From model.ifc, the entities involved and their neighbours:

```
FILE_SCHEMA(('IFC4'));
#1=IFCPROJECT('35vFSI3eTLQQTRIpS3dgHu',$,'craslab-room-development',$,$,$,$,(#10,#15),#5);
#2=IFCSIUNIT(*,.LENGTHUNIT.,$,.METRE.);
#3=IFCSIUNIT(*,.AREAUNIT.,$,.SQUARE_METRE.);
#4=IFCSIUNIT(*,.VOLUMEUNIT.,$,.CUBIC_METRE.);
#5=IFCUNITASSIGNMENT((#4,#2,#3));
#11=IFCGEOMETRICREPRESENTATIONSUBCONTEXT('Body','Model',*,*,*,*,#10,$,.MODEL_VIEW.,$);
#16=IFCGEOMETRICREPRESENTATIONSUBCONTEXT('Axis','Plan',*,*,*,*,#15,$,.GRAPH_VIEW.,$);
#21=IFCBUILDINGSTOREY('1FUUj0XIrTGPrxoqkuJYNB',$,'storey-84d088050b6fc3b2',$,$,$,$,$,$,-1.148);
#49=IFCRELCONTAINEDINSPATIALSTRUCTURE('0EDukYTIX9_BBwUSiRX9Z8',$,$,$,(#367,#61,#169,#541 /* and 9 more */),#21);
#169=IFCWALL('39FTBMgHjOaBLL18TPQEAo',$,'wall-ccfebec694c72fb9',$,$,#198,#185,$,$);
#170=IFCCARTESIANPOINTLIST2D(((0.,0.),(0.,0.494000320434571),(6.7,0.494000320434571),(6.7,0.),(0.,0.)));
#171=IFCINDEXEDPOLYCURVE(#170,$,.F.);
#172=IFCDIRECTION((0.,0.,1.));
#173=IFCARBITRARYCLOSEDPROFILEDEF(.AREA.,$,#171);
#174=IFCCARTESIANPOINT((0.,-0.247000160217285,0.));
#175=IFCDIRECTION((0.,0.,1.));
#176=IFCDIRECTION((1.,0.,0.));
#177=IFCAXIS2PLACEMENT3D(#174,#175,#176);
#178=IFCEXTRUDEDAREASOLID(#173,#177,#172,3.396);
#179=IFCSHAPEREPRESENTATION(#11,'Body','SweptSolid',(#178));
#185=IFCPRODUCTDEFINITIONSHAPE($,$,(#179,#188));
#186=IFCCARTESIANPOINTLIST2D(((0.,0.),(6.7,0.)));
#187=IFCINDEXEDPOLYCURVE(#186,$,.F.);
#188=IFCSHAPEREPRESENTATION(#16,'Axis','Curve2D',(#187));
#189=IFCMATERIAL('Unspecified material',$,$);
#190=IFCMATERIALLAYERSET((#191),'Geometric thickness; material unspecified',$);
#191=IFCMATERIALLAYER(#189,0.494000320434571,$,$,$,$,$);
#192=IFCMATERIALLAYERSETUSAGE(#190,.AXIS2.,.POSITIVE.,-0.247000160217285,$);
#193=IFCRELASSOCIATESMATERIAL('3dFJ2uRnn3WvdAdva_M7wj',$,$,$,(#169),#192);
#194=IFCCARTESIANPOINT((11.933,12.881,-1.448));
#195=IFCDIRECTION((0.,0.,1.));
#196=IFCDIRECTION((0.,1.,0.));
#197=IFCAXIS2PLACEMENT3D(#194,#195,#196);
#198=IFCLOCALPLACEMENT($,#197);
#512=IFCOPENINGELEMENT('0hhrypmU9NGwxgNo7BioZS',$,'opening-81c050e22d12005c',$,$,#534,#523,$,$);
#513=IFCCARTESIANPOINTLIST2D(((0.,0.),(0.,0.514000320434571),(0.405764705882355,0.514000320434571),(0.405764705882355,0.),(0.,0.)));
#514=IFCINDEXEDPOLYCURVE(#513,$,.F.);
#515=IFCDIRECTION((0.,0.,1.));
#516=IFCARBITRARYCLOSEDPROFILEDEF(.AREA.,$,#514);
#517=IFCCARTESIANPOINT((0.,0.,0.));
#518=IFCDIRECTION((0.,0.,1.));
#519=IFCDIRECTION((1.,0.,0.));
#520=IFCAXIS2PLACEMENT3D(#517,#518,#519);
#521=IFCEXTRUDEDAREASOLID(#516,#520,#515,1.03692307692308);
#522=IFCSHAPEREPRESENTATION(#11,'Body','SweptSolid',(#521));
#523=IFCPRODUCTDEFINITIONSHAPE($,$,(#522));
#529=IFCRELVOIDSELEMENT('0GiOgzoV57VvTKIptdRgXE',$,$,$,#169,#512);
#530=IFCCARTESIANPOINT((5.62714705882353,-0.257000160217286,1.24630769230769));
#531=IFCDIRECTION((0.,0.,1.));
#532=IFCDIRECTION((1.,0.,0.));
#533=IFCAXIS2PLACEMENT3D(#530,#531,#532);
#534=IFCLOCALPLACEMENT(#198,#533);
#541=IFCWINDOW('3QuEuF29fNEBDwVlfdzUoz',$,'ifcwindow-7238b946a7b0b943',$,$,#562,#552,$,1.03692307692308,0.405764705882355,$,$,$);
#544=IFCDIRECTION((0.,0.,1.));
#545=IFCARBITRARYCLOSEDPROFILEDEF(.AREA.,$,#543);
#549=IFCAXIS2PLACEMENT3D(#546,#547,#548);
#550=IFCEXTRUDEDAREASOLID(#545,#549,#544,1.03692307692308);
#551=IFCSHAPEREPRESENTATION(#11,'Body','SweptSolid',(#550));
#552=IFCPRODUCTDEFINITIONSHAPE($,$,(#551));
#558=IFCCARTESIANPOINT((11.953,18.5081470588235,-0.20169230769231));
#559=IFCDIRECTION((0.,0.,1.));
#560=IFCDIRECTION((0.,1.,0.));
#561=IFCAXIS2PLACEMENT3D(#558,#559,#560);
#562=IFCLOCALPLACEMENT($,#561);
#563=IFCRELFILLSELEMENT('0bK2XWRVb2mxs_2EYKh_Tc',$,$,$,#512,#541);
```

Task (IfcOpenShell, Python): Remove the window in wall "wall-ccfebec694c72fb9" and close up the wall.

```python
import ifcopenshell
import ifcopenshell.api.feature
import ifcopenshell.api.root
import ifcopenshell.geom
import ifcopenshell.util.shape

model = ifcopenshell.open("model.ifc")
settings = ifcopenshell.geom.settings()


def volume(element):
    """Net volume in cubic metres, openings subtracted."""
    shape = ifcopenshell.geom.create_shape(settings, element)
    return ifcopenshell.util.shape.get_volume(shape.geometry)


window = model.by_guid("3QuEuF29fNEBDwVlfdzUoz")
opening = window.FillsVoids[0].RelatingOpeningElement
wall = opening.VoidsElements[0].RelatingBuildingElement
before = volume(wall)

ifcopenshell.api.root.remove_product(model, product=window)
ifcopenshell.api.feature.remove_feature(model, feature=opening)

after = volume(wall)

print(f"wall volume {before:.3f} -> {after:.3f} m3")

model.write("model_v2.ifc")
```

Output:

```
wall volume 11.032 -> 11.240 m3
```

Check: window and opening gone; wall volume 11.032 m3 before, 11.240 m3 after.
